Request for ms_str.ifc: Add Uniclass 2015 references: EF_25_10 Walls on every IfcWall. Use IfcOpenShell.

First a look at what the model holds.

```python
import ifcopenshell

model = ifcopenshell.open("ms_str.ifc")
print(model.schema)
print("classifications:", [c.Name for c in model.by_type("IfcClassification")])
for ifc_class in ("IfcDoor", "IfcRoof", "IfcStair", "IfcWall", "IfcWindow"):
    print(ifc_class, len(model.by_type(ifc_class)))
```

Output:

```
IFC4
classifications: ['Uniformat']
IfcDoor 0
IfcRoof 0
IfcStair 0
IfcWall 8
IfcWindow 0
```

```python
import ifcopenshell
import ifcopenshell.api.classification

model = ifcopenshell.open("ms_str.ifc")

system = ifcopenshell.api.classification.add_classification(model, classification="Uniclass 2015")

codes = {
    "IfcWall": ("EF_25_10", "Walls"),
}
for ifc_class, (code, name) in codes.items():
    products = model.by_type(ifc_class)
    ifcopenshell.api.classification.add_reference(
        model, products=products, classification=system, identification=code, name=name
    )
    print(code, len(products))

model.write("ms_str_rev.ifc")
```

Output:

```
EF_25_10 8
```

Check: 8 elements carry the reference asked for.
